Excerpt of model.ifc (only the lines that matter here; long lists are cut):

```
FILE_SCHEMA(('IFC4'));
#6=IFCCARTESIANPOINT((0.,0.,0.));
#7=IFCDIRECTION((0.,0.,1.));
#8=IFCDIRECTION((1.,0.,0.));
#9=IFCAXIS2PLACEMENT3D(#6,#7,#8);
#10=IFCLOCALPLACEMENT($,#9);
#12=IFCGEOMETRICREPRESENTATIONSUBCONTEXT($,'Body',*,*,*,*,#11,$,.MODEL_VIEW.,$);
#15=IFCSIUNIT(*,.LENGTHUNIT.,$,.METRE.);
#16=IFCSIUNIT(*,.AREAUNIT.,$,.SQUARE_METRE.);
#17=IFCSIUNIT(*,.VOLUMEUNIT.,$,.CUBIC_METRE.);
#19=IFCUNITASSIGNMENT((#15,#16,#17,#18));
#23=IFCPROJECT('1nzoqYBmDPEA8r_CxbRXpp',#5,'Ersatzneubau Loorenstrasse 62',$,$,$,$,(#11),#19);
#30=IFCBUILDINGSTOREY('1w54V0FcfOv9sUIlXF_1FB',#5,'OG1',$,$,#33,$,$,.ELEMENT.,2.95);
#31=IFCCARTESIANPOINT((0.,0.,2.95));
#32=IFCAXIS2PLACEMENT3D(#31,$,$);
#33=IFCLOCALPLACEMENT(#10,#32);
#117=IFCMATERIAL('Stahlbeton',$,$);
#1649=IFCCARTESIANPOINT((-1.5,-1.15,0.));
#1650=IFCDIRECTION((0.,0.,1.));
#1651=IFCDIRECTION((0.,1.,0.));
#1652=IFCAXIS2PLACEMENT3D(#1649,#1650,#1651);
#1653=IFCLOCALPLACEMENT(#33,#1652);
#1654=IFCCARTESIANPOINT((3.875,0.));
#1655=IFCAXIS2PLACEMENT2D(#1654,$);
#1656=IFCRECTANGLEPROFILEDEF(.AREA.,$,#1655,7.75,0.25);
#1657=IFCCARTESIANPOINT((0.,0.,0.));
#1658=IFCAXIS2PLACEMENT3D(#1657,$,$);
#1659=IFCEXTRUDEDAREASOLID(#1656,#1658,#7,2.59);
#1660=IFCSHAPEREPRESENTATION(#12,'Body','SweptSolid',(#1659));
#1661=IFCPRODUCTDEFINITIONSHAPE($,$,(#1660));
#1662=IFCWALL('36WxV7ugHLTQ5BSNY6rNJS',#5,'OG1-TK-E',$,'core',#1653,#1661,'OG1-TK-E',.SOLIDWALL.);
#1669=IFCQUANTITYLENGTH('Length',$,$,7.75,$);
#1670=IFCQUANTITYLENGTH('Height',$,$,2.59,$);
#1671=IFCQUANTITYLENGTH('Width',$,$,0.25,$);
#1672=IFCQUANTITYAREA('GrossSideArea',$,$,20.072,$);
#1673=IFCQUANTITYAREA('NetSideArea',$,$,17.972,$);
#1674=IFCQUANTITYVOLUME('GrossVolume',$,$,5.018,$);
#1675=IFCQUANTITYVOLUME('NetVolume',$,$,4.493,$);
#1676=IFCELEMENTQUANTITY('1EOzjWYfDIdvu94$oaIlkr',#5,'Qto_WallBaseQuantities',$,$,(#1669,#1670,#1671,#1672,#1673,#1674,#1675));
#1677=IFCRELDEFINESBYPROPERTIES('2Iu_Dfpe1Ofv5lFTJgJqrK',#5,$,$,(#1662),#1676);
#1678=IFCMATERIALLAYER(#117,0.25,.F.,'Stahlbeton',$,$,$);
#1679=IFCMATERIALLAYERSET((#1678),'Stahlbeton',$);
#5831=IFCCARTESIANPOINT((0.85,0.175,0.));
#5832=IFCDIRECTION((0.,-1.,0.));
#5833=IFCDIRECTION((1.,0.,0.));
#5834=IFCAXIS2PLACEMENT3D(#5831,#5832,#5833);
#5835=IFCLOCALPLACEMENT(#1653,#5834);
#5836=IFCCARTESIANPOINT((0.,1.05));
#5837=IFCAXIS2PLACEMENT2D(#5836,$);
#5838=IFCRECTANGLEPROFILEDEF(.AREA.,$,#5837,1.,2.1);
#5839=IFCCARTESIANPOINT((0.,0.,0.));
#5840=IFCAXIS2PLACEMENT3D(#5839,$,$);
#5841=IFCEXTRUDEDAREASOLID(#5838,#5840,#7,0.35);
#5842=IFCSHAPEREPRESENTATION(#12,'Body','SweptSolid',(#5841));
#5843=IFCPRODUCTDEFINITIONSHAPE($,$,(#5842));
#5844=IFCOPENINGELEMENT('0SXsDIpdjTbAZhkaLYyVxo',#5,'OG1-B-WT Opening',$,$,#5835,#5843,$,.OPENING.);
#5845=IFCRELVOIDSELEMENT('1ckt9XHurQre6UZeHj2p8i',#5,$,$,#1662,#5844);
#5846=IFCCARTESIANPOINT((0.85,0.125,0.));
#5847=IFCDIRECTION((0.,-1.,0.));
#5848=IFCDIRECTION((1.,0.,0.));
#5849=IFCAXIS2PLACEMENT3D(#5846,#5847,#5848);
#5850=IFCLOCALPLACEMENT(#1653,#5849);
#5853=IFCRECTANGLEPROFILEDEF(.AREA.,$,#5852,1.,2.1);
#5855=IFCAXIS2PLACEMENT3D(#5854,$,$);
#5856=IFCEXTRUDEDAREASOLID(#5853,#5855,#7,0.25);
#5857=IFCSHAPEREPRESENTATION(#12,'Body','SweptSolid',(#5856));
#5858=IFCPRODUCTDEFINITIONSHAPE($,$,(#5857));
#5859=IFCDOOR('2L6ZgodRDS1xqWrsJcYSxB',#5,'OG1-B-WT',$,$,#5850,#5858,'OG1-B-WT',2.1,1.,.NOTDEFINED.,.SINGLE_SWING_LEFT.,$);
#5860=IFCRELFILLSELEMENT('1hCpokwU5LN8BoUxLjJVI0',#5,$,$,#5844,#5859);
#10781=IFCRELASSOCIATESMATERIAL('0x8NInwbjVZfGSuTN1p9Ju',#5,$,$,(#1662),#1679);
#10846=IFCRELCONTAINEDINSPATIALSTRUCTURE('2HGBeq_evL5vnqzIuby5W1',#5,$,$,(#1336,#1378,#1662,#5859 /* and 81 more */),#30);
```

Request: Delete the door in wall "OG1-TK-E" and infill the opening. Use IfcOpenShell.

```python
import ifcopenshell
import ifcopenshell.api.feature
import ifcopenshell.api.pset
import ifcopenshell.api.root
import ifcopenshell.geom
import ifcopenshell.util.element
import ifcopenshell.util.shape
import ifcopenshell.util.unit

model = ifcopenshell.open("model.ifc")
area_scale = ifcopenshell.util.unit.calculate_unit_scale(model, "AREAUNIT")
volume_scale = ifcopenshell.util.unit.calculate_unit_scale(model, "VOLUMEUNIT")
settings = ifcopenshell.geom.settings()


def volume(element):
    """Net volume in cubic metres, openings subtracted."""
    shape = ifcopenshell.geom.create_shape(settings, element)
    return ifcopenshell.util.shape.get_volume(shape.geometry)


door = model.by_id(5859)
opening = door.FillsVoids[0].RelatingOpeningElement
wall = opening.VoidsElements[0].RelatingBuildingElement
before = volume(wall)

ifcopenshell.api.root.remove_product(model, product=door)
ifcopenshell.api.feature.remove_feature(model, feature=opening)

after = volume(wall)
thickness = 0.25  # wall thickness in metres

# Update the wall's stored quantities.
qto = model.by_id(ifcopenshell.util.element.get_pset(wall, "Qto_WallBaseQuantities", should_inherit=False)["id"])
ifcopenshell.api.pset.edit_qto(model, qto=qto, properties={
    "NetSideArea": after / thickness / area_scale,
    "NetVolume": after / volume_scale,
})

print(f"wall volume {before:.3f} -> {after:.3f} m3")

model.write("model_edited.ifc")
```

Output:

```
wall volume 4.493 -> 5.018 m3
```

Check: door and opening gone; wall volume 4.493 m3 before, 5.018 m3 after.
